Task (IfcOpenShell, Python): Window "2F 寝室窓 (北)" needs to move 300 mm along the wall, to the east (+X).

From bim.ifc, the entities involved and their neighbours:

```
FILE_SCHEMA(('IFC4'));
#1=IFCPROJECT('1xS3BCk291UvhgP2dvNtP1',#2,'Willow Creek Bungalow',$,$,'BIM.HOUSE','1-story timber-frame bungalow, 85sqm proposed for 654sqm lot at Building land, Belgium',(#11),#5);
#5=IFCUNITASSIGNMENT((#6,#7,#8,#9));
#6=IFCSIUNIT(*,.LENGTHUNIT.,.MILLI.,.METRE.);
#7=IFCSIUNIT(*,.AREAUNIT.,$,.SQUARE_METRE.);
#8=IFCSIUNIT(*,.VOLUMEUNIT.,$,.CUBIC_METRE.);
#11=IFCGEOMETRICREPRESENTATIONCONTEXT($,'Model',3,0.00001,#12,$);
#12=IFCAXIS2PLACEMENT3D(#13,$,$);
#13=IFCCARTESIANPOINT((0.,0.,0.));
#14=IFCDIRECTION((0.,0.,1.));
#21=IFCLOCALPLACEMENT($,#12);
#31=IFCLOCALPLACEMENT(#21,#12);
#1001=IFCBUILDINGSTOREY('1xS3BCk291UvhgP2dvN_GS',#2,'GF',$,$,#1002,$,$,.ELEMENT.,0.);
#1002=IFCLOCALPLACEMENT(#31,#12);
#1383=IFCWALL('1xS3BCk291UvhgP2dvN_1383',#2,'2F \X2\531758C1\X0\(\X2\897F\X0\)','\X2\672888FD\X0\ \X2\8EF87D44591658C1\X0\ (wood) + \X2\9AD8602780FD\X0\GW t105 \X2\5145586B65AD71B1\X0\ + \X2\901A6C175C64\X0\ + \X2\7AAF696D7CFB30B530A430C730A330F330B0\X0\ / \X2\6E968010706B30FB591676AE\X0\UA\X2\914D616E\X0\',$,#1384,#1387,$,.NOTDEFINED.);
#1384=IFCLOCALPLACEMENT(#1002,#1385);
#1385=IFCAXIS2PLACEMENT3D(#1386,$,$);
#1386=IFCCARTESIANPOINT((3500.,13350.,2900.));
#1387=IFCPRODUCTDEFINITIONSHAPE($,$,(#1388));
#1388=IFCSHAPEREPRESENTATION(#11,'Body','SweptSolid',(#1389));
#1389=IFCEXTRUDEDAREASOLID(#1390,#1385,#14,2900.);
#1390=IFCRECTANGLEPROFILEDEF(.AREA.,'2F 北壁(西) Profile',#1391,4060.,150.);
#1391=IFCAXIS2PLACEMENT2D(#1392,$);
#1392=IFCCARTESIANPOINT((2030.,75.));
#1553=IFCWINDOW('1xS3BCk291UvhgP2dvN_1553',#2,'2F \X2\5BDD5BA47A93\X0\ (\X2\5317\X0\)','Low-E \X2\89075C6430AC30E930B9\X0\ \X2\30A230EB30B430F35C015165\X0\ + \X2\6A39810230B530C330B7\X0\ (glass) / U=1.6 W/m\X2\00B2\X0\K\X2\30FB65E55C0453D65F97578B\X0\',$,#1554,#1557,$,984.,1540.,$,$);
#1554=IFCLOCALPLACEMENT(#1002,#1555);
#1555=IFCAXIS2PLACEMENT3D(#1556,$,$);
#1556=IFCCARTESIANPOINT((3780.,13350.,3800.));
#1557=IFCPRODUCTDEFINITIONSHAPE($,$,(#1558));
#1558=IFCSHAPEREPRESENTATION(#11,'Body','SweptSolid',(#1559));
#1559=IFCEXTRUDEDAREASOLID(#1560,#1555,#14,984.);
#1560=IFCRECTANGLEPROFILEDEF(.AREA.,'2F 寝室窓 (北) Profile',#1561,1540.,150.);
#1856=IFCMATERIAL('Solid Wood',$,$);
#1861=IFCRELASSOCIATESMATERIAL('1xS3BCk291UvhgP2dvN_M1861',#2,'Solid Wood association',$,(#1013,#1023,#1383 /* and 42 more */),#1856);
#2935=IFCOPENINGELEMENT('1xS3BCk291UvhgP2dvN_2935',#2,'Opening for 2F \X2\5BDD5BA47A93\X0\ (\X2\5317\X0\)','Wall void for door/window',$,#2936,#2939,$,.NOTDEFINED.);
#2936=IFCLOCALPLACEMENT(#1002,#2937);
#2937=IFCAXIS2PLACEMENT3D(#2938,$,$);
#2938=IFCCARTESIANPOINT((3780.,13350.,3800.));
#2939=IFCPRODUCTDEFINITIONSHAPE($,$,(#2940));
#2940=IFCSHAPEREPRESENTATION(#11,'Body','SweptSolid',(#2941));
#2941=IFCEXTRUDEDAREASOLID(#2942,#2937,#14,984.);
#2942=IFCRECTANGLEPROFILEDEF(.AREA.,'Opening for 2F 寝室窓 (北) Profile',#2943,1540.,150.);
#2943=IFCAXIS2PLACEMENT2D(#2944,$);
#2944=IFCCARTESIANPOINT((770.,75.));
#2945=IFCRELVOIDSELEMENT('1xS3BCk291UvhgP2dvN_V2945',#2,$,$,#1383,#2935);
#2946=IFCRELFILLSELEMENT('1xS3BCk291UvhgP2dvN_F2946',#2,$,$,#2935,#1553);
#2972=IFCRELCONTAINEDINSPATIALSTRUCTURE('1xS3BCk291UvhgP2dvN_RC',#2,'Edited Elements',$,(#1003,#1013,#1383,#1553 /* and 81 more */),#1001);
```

```python
import ifcopenshell
import ifcopenshell.api.geometry
import ifcopenshell.util.placement
import ifcopenshell.util.unit

model = ifcopenshell.open("bim.ifc")
unit_scale = ifcopenshell.util.unit.calculate_unit_scale(model)

window = model.by_guid("1xS3BCk291UvhgP2dvN_1553")
opening = window.FillsVoids[0].RelatingOpeningElement
wall = opening.VoidsElements[0].RelatingBuildingElement

wall_matrix = ifcopenshell.util.placement.get_local_placement(wall.ObjectPlacement)
shift = wall_matrix[:3, 0] * 0.3 / unit_scale
before = ifcopenshell.util.placement.get_local_placement(window.ObjectPlacement)[:3, 3].copy()

# The window is not placed relative to its opening, so move both.
for product in (opening, window):
    matrix = ifcopenshell.util.placement.get_local_placement(product.ObjectPlacement)
    matrix[:3, 3] += shift
    ifcopenshell.api.geometry.edit_object_placement(model, product=product, matrix=matrix, is_si=False)

after = ifcopenshell.util.placement.get_local_placement(window.ObjectPlacement)[:3, 3]
print("window moved by", (after - before).round(3) + 0.0)

model.write("bim_v2.ifc")
```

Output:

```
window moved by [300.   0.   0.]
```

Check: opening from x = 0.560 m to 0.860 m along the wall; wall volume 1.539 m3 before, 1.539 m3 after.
